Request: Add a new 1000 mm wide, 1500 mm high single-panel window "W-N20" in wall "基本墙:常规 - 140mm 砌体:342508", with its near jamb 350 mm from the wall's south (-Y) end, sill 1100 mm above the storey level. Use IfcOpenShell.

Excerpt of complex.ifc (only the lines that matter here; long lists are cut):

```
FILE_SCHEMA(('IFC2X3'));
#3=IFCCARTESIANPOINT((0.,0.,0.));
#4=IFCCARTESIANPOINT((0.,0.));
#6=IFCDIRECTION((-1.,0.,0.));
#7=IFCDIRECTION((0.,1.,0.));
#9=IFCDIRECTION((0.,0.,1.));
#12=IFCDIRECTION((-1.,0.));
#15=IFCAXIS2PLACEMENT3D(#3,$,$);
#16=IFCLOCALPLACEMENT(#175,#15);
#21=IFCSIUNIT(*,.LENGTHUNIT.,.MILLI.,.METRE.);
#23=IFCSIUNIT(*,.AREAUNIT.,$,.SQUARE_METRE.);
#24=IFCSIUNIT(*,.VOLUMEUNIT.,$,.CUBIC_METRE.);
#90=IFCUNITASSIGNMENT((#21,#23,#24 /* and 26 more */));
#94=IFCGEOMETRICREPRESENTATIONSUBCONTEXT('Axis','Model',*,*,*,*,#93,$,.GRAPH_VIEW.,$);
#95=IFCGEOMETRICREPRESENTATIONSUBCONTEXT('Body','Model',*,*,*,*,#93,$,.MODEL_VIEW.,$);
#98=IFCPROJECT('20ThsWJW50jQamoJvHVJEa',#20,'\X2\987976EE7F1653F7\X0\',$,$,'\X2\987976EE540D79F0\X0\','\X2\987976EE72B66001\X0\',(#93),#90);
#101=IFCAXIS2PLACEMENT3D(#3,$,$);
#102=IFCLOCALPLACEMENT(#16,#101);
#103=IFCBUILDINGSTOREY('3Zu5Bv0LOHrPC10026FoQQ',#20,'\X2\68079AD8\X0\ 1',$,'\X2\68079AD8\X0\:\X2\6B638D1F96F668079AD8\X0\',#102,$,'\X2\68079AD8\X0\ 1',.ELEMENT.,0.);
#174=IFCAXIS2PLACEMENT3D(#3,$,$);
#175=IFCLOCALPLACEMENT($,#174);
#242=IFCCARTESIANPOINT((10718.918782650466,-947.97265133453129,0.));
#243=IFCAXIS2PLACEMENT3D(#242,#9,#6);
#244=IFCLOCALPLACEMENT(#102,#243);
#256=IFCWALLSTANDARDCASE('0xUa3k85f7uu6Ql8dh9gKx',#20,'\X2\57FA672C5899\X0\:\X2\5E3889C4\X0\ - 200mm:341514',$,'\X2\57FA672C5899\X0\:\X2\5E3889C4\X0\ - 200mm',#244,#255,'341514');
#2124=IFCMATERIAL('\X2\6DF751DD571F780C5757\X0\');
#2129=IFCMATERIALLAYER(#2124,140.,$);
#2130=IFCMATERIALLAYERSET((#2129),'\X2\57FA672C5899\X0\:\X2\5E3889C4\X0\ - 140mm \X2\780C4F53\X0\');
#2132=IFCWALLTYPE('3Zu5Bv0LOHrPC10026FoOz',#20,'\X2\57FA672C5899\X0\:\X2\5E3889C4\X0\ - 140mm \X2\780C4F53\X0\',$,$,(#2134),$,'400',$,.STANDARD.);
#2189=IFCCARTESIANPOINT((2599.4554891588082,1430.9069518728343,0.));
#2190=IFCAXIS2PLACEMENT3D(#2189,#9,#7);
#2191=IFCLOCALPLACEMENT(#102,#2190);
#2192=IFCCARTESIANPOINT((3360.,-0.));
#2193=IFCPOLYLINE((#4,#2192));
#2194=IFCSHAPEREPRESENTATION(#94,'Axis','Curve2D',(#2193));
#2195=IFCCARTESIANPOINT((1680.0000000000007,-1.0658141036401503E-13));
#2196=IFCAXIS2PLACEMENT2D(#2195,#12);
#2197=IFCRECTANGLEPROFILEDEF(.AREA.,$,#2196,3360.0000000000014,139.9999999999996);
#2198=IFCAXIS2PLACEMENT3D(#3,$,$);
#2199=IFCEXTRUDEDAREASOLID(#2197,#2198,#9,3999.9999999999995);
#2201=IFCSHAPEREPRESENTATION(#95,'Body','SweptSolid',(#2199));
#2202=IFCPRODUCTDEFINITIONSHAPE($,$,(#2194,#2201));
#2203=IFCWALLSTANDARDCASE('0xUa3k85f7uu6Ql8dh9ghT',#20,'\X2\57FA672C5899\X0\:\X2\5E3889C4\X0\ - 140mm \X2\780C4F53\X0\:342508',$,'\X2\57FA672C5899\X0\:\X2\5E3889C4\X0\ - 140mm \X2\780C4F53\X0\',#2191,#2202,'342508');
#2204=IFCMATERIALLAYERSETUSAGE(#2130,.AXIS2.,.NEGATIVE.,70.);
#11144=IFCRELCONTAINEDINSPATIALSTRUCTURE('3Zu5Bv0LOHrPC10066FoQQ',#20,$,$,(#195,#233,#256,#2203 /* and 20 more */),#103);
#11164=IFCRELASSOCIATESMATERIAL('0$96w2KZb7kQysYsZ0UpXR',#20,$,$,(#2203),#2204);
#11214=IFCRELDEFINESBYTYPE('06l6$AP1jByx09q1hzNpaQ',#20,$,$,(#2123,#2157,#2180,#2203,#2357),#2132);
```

```python
import numpy as np
import ifcopenshell
import ifcopenshell.api.feature
import ifcopenshell.api.geometry
import ifcopenshell.api.root
import ifcopenshell.api.spatial
import ifcopenshell.api.type
import ifcopenshell.geom
import ifcopenshell.util.element
import ifcopenshell.util.placement
import ifcopenshell.util.representation
import ifcopenshell.util.shape
import ifcopenshell.util.unit

model = ifcopenshell.open("complex.ifc")
unit_scale = ifcopenshell.util.unit.calculate_unit_scale(model)
settings = ifcopenshell.geom.settings()


def volume(element):
    """Net volume in cubic metres, openings subtracted."""
    shape = ifcopenshell.geom.create_shape(settings, element)
    return ifcopenshell.util.shape.get_volume(shape.geometry)


wall = model.by_id(2203)
storey = ifcopenshell.util.element.get_container(wall, ifc_class="IfcBuildingStorey")
context = ifcopenshell.util.representation.get_context(model, "Model", "Body", "MODEL_VIEW")
before = volume(wall)

width, height, from_end, sill = 1, 1.5, 0.35, 1.1  # metres

# The wall runs along its own X axis, and the end named is its -X end.
wall_shape = ifcopenshell.geom.create_shape(settings, wall)
x, y, z = ifcopenshell.util.shape.get_vertices(wall_shape.geometry).T
start = x.min() + from_end
face, thickness = float(y.min()), float(y.max() - y.min())
wall_matrix = ifcopenshell.util.placement.get_local_placement(wall.ObjectPlacement)
level = ifcopenshell.util.placement.get_local_placement(storey.ObjectPlacement)[2, 3]


def in_wall(x, y):
    """Placement at x, y metres in the wall's axes, at sill height."""
    matrix = wall_matrix.copy()
    matrix[:, 3] = wall_matrix @ np.array([x / unit_scale, y / unit_scale, 0.0, 1.0])
    matrix[2, 3] = level + sill / unit_scale
    return matrix


# Opening: a box that overshoots both wall faces by 50 mm.
opening = ifcopenshell.api.root.create_entity(model, ifc_class="IfcOpeningElement")
box = ifcopenshell.api.geometry.add_wall_representation(
    model, context=context, length=width, height=height, thickness=thickness + 0.1
)
ifcopenshell.api.geometry.assign_representation(model, product=opening, representation=box)
ifcopenshell.api.geometry.edit_object_placement(model, product=opening, matrix=in_wall(start, face - 0.05), is_si=False)
ifcopenshell.api.feature.add_feature(model, feature=opening, element=wall)

window = ifcopenshell.api.root.create_entity(model, ifc_class="IfcWindow", name="W-N20")
window.OverallWidth, window.OverallHeight = width / unit_scale, height / unit_scale
body = ifcopenshell.api.geometry.add_window_representation(
    model,
    context=context,
    overall_width=window.OverallWidth,
    overall_height=window.OverallHeight,
    partition_type="SINGLE_PANEL",
)
ifcopenshell.api.geometry.assign_representation(model, product=window, representation=body)
ifcopenshell.api.spatial.assign_container(model, products=[window], relating_structure=storey)
fills = ifcopenshell.api.feature.add_filling(model, opening=opening, element=window)
fills.OwnerHistory = window.OwnerHistory  # required in IFC2X3

# IFC2X3 keeps the operation on the window style.
style = ifcopenshell.api.root.create_entity(model, ifc_class="IfcWindowStyle", name="W-N20")
style.OperationType, style.ConstructionType = "SINGLE_PANEL", "NOTDEFINED"
style.ParameterTakesPrecedence = style.Sizeable = False
ifcopenshell.api.type.assign_type(model, related_objects=[window], relating_type=style)

# Centre the window in the wall's thickness.
ifcopenshell.api.geometry.edit_object_placement(model, product=window, matrix=in_wall(start, face), is_si=False)
window_shape = ifcopenshell.geom.create_shape(settings, window)
depth = ifcopenshell.util.shape.get_vertices(window_shape.geometry)[:, 1]
offset = face + thickness / 2 - (depth.min() + depth.max()) / 2
ifcopenshell.api.geometry.edit_object_placement(model, product=window, matrix=in_wall(start, offset), is_si=False)

after = volume(wall)

print(f"wall volume {before:.3f} -> {after:.3f} m3")

model.write("complex_rev.ifc")
```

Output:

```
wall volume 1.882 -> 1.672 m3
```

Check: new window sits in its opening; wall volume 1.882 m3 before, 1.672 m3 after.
